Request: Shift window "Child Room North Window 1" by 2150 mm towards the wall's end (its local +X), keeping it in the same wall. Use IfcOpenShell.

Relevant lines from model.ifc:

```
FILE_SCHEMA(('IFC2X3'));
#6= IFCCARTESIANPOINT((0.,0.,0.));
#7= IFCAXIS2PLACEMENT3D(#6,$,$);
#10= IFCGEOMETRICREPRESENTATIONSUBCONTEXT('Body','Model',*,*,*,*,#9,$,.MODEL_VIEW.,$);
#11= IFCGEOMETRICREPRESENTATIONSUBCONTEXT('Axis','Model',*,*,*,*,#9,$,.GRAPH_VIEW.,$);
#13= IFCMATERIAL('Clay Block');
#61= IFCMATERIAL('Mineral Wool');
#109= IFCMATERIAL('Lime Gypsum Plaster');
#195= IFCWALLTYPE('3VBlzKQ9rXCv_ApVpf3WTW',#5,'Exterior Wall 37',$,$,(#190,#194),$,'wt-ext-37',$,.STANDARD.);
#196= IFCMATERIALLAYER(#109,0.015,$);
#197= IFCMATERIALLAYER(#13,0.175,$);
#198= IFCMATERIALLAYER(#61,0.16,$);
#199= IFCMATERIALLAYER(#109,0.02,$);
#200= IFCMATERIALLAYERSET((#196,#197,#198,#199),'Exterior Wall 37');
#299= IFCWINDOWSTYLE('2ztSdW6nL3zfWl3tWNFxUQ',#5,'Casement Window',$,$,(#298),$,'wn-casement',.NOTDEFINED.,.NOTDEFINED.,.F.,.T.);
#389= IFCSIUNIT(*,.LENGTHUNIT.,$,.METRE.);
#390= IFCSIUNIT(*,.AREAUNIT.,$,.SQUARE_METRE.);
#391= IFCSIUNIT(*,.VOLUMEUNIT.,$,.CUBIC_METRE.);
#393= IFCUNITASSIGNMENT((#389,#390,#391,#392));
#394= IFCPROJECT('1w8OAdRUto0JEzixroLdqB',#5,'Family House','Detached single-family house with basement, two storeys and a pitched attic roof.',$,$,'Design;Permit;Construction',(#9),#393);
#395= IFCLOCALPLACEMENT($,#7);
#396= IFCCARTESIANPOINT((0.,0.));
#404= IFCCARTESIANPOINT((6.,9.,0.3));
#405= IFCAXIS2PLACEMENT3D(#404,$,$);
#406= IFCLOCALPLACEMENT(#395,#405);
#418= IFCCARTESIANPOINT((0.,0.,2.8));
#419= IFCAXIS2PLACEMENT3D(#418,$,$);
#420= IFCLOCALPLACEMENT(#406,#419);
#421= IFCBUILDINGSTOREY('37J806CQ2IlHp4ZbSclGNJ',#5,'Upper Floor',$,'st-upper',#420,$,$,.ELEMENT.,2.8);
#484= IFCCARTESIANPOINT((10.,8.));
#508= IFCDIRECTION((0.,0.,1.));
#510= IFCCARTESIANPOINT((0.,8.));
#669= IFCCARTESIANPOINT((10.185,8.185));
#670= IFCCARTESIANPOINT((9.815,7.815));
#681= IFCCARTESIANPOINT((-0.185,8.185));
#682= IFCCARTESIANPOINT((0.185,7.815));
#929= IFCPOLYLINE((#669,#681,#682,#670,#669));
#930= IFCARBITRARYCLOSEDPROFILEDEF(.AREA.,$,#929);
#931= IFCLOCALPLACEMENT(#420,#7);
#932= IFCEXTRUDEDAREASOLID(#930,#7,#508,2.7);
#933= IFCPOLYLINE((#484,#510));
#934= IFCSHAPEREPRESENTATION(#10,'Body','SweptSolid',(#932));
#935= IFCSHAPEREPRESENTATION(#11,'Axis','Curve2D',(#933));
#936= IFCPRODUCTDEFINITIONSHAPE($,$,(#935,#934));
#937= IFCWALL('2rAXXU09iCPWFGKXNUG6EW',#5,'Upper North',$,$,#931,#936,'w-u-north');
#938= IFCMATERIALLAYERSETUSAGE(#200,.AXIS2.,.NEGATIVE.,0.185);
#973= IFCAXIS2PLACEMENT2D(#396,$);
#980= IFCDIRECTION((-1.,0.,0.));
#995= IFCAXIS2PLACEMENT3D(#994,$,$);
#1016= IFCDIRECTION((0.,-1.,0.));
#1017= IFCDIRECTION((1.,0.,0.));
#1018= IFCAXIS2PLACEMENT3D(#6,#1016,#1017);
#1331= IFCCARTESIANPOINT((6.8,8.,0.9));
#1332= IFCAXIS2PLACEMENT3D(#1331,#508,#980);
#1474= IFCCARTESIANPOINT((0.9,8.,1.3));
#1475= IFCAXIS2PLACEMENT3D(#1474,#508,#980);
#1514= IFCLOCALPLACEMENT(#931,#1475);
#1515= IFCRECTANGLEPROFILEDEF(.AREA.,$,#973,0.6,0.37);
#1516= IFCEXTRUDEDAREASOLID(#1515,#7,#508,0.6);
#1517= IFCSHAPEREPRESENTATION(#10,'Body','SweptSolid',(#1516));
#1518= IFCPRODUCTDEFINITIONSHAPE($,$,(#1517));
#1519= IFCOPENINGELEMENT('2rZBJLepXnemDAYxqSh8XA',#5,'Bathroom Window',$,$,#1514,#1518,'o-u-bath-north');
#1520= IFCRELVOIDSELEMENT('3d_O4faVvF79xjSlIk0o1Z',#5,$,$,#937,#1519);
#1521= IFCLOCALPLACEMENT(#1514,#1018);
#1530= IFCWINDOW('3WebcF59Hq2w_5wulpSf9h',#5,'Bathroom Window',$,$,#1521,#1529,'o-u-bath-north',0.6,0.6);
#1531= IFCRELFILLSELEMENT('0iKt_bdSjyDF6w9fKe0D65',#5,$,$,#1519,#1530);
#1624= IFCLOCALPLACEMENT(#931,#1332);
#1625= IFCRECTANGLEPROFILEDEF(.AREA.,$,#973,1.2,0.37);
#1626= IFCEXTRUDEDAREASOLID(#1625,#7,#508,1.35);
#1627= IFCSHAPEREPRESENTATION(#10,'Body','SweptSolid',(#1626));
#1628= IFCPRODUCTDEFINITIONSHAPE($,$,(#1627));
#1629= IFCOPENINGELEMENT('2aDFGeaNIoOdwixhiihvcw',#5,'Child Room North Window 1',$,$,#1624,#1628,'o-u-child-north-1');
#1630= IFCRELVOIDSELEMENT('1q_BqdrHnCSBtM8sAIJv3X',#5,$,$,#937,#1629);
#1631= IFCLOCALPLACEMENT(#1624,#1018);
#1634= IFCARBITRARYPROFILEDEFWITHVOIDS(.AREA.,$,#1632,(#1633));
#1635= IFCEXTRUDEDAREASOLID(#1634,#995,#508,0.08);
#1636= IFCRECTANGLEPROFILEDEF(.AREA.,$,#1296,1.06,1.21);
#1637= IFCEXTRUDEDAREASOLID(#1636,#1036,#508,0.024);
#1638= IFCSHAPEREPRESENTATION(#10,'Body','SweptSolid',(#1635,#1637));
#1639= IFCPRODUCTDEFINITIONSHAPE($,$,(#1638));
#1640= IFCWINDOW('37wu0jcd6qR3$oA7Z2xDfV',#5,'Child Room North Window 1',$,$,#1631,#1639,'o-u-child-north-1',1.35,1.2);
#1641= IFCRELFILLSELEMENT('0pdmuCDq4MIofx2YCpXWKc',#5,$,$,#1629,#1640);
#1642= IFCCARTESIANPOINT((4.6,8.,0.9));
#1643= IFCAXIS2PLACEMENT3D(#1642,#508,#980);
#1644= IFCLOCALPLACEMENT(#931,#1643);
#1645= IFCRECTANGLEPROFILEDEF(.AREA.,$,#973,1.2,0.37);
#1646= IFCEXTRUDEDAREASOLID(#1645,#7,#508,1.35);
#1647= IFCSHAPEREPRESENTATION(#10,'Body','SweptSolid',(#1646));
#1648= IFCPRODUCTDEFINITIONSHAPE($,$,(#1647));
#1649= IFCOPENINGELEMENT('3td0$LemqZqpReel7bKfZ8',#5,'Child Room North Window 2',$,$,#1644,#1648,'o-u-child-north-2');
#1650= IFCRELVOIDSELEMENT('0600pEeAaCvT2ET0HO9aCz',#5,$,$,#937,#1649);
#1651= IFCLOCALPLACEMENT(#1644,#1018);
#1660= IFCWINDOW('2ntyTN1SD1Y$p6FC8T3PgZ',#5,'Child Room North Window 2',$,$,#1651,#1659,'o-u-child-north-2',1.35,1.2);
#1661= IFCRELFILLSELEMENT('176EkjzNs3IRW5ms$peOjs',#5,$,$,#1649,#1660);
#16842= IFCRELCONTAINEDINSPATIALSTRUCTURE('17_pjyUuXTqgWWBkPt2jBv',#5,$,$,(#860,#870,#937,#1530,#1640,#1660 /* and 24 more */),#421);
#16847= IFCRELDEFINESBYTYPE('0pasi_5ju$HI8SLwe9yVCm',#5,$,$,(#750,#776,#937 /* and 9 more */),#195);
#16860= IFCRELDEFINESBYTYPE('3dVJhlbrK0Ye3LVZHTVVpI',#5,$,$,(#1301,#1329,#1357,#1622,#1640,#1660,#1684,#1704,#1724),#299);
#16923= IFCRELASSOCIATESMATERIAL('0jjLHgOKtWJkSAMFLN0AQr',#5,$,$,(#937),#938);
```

```python
import ifcopenshell
import ifcopenshell.api.geometry
import ifcopenshell.util.placement
import ifcopenshell.util.unit

model = ifcopenshell.open("model.ifc")
unit_scale = ifcopenshell.util.unit.calculate_unit_scale(model)

window = model.by_guid("37wu0jcd6qR3$oA7Z2xDfV")
opening = window.FillsVoids[0].RelatingOpeningElement
wall = opening.VoidsElements[0].RelatingBuildingElement

wall_matrix = ifcopenshell.util.placement.get_local_placement(wall.ObjectPlacement)
shift = wall_matrix[:3, 0] * 2.15 / unit_scale
before = ifcopenshell.util.placement.get_local_placement(window.ObjectPlacement)[:3, 3].copy()

# The window is placed relative to its opening, so it follows when the opening moves.
matrix = ifcopenshell.util.placement.get_local_placement(opening.ObjectPlacement)
matrix[:3, 3] += shift
ifcopenshell.api.geometry.edit_object_placement(
    model, product=opening, matrix=matrix, is_si=False, should_transform_children=True
)

after = ifcopenshell.util.placement.get_local_placement(window.ObjectPlacement)[:3, 3]
print("window moved by", (after - before).round(3) + 0.0)

model.write("model_rev.ifc")
```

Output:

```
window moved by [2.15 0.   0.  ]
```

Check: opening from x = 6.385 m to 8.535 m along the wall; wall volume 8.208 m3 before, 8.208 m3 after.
